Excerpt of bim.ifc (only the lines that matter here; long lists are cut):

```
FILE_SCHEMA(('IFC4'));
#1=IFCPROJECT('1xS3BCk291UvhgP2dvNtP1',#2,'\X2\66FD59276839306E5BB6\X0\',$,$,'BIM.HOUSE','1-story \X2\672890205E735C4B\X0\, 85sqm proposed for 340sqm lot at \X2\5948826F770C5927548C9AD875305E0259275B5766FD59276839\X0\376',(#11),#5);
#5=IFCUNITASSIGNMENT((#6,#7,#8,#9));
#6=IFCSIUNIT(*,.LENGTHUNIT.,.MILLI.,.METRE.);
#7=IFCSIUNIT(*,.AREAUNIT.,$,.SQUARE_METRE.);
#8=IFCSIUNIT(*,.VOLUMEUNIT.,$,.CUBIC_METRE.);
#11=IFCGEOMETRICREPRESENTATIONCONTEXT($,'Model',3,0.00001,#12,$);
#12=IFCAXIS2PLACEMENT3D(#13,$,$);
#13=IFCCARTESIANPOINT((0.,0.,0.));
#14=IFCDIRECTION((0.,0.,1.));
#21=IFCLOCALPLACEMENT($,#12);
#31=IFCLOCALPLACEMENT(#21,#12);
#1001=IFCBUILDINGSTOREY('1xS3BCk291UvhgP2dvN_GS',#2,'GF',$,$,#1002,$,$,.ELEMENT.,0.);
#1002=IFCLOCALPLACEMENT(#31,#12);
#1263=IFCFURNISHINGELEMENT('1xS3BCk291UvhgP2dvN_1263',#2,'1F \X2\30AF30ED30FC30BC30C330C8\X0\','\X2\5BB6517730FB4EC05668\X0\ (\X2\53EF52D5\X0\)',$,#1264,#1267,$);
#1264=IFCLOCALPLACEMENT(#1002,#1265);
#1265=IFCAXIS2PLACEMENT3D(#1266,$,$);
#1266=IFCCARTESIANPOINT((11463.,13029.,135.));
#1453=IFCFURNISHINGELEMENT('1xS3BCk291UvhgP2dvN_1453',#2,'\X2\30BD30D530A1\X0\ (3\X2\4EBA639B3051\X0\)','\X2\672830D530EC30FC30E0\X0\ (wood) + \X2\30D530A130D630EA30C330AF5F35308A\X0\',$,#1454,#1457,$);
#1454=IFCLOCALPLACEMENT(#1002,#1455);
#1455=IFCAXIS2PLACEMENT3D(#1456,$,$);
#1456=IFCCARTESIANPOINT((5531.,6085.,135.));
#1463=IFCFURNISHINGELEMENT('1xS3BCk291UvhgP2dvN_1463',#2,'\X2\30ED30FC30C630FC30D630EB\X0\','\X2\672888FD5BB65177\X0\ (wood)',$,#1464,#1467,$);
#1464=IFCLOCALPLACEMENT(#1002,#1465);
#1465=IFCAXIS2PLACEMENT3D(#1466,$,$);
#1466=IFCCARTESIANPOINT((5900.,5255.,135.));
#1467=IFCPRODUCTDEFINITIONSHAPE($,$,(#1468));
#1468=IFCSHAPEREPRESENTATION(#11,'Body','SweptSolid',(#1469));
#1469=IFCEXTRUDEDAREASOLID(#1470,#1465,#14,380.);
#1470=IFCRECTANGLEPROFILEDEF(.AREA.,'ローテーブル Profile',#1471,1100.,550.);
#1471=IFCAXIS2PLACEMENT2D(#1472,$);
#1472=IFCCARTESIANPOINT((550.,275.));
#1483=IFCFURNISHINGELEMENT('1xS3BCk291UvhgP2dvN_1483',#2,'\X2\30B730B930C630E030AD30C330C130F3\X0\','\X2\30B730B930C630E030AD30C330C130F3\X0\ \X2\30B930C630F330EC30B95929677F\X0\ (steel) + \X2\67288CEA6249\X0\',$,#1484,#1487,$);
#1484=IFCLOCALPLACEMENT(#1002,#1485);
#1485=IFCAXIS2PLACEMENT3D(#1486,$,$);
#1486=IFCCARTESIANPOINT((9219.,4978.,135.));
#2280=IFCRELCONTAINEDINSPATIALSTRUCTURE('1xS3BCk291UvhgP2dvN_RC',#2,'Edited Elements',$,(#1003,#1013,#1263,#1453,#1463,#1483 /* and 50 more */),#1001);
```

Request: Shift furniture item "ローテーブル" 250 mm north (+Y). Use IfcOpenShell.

```python
import ifcopenshell
import ifcopenshell.api.geometry
import ifcopenshell.util.placement
import ifcopenshell.util.unit

model = ifcopenshell.open("bim.ifc")
unit_scale = ifcopenshell.util.unit.calculate_unit_scale(model)

item = model.by_guid("1xS3BCk291UvhgP2dvN_1463")
matrix = ifcopenshell.util.placement.get_local_placement(item.ObjectPlacement)
matrix[1, 3] += 0.25 / unit_scale
ifcopenshell.api.geometry.edit_object_placement(model, product=item, matrix=matrix, is_si=False)

print(ifcopenshell.util.placement.get_local_placement(item.ObjectPlacement).round(3) + 0.0)

model.write("bim_v2.ifc")
```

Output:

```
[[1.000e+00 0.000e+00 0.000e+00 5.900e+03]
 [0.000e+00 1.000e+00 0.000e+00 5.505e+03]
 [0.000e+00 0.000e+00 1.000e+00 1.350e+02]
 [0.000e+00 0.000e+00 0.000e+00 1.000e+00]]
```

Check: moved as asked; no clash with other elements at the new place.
